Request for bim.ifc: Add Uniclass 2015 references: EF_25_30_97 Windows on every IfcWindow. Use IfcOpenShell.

First a look at what the model holds.

```python
import ifcopenshell

model = ifcopenshell.open("bim.ifc")
print(model.schema)
print("classifications:", [c.Name for c in model.by_type("IfcClassification")])
for ifc_class in ("IfcDoor", "IfcRoof", "IfcStair", "IfcWall", "IfcWindow"):
    print(ifc_class, len(model.by_type(ifc_class)))
```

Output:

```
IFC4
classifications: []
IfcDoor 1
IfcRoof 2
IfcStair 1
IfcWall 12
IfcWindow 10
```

```python
import ifcopenshell
import ifcopenshell.api.classification

model = ifcopenshell.open("bim.ifc")

system = ifcopenshell.api.classification.add_classification(model, classification="Uniclass 2015")

codes = {
    "IfcWindow": ("EF_25_30_97", "Windows"),
}
for ifc_class, (code, name) in codes.items():
    products = model.by_type(ifc_class)
    ifcopenshell.api.classification.add_reference(
        model, products=products, classification=system, identification=code, name=name
    )
    print(code, len(products))

model.write("bim_rev.ifc")
```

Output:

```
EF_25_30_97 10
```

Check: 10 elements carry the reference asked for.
